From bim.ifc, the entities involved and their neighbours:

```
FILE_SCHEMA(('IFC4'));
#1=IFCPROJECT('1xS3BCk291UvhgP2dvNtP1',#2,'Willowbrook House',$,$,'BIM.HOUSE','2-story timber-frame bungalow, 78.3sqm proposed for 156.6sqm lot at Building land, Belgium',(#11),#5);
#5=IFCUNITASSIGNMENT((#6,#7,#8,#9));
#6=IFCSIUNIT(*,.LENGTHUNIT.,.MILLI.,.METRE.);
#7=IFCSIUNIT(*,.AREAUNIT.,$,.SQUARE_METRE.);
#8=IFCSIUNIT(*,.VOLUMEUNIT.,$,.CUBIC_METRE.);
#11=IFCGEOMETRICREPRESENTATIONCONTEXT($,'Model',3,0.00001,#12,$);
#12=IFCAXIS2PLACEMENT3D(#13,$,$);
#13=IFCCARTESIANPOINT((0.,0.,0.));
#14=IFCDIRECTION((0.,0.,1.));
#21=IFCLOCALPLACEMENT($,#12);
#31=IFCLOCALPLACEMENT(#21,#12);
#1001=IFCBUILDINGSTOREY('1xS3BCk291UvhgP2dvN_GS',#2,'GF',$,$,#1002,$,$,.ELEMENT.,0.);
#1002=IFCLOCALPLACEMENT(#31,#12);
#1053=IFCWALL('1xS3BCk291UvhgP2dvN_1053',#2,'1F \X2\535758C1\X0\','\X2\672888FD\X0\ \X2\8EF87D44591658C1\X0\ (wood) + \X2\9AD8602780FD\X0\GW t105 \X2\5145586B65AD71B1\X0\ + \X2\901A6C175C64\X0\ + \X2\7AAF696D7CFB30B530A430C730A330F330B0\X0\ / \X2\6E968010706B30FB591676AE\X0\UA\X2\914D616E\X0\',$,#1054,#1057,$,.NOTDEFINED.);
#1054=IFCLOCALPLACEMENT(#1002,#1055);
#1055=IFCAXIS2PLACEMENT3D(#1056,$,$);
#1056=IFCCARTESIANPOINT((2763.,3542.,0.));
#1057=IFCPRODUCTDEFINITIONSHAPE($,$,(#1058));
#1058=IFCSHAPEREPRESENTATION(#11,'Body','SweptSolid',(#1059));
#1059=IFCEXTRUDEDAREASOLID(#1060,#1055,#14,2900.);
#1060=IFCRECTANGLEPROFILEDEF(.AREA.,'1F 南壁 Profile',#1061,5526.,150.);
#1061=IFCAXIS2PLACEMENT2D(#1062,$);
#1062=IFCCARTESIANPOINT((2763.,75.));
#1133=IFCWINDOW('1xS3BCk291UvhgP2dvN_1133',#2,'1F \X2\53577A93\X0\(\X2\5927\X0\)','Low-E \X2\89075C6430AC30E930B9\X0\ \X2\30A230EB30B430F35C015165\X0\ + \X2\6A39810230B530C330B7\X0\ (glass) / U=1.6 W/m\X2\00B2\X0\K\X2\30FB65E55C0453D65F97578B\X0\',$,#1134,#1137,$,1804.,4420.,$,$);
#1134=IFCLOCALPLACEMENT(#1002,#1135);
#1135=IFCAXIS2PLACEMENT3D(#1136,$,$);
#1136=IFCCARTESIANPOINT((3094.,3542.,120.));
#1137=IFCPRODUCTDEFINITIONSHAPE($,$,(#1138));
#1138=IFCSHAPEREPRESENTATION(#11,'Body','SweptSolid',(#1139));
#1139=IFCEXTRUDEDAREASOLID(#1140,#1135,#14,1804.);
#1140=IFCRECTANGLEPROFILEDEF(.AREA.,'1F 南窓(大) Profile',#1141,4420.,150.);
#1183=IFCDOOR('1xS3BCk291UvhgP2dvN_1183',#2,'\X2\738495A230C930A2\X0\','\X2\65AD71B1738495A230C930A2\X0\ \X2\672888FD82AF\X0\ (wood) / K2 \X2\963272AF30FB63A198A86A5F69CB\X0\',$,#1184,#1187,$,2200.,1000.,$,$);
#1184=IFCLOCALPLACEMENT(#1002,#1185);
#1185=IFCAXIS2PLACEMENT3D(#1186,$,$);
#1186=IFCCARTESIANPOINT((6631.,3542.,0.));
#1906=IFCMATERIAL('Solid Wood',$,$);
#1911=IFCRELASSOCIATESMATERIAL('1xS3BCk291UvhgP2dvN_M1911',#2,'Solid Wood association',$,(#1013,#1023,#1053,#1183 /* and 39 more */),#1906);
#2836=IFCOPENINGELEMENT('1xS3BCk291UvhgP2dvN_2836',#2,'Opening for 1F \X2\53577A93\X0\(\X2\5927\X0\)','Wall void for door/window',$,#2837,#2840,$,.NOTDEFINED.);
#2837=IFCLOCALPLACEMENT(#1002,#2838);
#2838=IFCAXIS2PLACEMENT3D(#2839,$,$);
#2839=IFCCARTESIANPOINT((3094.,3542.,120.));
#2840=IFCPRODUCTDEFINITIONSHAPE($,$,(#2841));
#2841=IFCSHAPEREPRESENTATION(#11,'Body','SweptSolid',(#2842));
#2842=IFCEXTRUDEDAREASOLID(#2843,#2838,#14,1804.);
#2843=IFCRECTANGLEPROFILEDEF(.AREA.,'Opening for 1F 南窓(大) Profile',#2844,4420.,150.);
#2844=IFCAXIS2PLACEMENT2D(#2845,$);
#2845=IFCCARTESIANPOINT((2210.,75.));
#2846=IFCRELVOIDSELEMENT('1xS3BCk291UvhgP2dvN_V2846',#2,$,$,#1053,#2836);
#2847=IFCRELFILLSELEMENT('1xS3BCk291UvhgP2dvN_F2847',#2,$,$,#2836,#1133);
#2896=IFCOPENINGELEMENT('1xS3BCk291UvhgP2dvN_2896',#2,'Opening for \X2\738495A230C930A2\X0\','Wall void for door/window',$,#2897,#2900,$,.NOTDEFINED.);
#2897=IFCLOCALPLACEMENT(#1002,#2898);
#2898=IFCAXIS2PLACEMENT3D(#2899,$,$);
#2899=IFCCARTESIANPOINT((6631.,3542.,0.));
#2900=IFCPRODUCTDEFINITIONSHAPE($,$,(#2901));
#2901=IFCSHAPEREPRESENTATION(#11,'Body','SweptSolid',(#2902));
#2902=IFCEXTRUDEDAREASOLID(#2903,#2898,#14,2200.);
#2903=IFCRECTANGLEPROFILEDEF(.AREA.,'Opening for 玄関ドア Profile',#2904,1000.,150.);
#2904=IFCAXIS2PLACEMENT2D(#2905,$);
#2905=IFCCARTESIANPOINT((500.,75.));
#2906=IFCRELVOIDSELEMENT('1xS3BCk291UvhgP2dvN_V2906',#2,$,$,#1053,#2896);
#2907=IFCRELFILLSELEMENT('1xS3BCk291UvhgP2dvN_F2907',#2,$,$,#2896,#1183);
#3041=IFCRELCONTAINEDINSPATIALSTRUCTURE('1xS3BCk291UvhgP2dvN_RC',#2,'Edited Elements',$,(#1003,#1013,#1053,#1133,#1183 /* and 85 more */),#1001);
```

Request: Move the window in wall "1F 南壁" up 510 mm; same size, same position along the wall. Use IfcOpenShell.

```python
import numpy as np
import ifcopenshell
import ifcopenshell.api.geometry
import ifcopenshell.util.placement
import ifcopenshell.util.unit

model = ifcopenshell.open("bim.ifc")
unit_scale = ifcopenshell.util.unit.calculate_unit_scale(model)

window = model.by_id(1133)
opening = window.FillsVoids[0].RelatingOpeningElement
dz = 0.51 / unit_scale

shift = np.array([0.0, 0.0, dz])
# The window is not placed relative to its opening, so move both.
for product in (opening, window):
    matrix = ifcopenshell.util.placement.get_local_placement(product.ObjectPlacement)
    matrix[:3, 3] += shift
    ifcopenshell.api.geometry.edit_object_placement(model, product=product, matrix=matrix, is_si=False)

print(f"moved by {dz * unit_scale:+.3f} m")

model.write("bim_updated.ifc")
```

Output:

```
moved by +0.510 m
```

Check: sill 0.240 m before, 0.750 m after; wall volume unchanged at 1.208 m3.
